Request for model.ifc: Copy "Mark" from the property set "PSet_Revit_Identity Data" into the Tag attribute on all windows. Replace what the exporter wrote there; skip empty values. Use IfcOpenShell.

First a look at what the model holds.

```python
import ifcopenshell
import ifcopenshell.util.element

model = ifcopenshell.open("model.ifc")
print(model.schema)
windows = model.by_type("IfcWindow")
print(len(windows), "windows")
for e in windows[:8]:
    source = ifcopenshell.util.element.get_pset(e, "PSet_Revit_Identity Data", "Mark")
    target = e.Tag
    print(e.id(), repr(source), repr(target), sep=" | ")
```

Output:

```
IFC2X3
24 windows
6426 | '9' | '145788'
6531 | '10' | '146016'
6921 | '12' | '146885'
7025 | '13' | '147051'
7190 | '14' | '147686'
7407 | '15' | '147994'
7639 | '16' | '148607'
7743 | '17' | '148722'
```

```python
import ifcopenshell
import ifcopenshell.util.element

model = ifcopenshell.open("model.ifc")

count = 0
for e in model.by_type("IfcWindow"):
    value = ifcopenshell.util.element.get_pset(e, "PSet_Revit_Identity Data", "Mark")
    current = e.Tag
    if not value or not value.strip() or current == value:
        continue
    e.Tag = value
    count += 1

print(count, "windows updated")

model.write("model_updated.ifc")
```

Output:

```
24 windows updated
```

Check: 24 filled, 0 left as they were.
